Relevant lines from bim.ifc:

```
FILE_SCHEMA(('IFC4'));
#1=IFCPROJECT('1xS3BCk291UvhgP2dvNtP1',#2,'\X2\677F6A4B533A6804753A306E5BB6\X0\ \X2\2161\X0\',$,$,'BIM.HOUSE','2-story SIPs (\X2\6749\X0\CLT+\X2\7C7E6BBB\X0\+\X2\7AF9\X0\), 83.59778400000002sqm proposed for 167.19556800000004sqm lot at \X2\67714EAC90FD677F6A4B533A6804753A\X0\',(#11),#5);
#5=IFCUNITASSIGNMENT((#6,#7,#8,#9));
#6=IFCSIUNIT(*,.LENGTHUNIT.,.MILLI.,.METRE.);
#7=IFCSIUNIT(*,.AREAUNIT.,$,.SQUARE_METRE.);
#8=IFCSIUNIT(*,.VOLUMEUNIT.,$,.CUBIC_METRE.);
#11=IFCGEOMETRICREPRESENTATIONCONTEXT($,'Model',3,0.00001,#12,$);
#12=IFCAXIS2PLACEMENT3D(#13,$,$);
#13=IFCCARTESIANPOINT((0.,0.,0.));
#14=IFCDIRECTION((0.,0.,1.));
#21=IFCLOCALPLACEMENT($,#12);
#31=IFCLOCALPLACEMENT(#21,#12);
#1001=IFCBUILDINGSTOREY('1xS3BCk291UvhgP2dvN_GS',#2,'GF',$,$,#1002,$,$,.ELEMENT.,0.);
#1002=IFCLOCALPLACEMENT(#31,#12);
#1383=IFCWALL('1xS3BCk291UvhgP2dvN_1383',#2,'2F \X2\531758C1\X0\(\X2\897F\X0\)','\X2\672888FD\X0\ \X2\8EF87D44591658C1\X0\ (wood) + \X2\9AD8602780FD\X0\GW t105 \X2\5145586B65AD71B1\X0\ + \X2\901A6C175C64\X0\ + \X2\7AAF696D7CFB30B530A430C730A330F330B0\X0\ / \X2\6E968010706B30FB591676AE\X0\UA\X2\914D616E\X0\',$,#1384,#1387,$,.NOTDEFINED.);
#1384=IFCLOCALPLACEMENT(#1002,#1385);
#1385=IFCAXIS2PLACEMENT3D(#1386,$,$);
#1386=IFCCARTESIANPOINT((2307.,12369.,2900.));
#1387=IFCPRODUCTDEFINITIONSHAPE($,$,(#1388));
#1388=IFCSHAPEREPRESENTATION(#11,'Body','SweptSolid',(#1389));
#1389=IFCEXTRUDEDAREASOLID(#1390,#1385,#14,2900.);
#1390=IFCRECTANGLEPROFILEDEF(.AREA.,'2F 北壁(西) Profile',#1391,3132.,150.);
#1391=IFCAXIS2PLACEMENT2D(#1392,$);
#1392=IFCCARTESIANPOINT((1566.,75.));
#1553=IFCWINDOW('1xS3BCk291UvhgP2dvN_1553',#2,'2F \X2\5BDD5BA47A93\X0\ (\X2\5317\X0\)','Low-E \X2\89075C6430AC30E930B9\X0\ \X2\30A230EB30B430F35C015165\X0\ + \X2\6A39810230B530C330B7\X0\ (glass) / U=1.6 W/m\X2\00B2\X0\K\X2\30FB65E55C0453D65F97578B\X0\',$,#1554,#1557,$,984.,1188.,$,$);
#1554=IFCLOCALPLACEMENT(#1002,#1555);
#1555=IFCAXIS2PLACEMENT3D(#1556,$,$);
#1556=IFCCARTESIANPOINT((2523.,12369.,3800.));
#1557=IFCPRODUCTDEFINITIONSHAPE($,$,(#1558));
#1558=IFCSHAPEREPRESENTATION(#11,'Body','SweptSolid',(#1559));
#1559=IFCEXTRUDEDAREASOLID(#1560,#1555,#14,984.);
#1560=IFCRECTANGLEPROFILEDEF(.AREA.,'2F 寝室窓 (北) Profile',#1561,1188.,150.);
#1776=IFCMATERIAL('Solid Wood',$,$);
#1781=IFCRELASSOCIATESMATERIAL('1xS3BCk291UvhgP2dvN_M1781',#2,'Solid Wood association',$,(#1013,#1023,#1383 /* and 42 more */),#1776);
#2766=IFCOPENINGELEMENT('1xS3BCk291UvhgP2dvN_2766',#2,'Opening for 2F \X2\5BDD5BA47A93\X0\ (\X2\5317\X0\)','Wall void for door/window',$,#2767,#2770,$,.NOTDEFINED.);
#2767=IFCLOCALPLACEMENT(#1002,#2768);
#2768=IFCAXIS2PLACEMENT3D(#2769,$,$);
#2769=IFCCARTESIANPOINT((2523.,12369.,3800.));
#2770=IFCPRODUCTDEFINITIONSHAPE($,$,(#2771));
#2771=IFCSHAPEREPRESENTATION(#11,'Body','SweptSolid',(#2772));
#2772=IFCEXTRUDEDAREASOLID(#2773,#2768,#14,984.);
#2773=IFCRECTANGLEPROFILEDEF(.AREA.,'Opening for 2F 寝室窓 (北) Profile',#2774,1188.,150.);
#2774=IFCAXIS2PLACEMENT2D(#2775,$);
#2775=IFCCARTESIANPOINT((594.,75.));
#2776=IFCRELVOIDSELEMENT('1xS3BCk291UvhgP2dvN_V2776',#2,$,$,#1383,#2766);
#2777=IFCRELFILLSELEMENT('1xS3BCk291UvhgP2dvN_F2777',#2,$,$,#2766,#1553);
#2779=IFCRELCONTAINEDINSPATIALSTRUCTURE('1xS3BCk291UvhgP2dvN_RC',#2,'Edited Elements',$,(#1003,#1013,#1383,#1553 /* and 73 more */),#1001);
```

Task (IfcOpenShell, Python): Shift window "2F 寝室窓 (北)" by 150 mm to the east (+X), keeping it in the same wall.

```python
import ifcopenshell
import ifcopenshell.api.geometry
import ifcopenshell.util.placement

model = ifcopenshell.open("bim.ifc")

window = model.by_guid("1xS3BCk291UvhgP2dvN_1553")
opening = window.FillsVoids[0].RelatingOpeningElement
wall = opening.VoidsElements[0].RelatingBuildingElement

wall_matrix = ifcopenshell.util.placement.get_local_placement(wall.ObjectPlacement)
shift = wall_matrix[:3, 0] * 150.0
before = ifcopenshell.util.placement.get_local_placement(window.ObjectPlacement)[:3, 3].copy()

# The window is not placed relative to its opening, so move both.
for product in (opening, window):
    matrix = ifcopenshell.util.placement.get_local_placement(product.ObjectPlacement)
    matrix[:3, 3] += shift
    ifcopenshell.api.geometry.edit_object_placement(model, product=product, matrix=matrix, is_si=False)

after = ifcopenshell.util.placement.get_local_placement(window.ObjectPlacement)[:3, 3]
print("window moved by", (after - before).round(3) + 0.0)

model.write("bim_rev.ifc")
```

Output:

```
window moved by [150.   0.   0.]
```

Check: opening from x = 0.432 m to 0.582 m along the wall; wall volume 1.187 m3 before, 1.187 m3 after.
